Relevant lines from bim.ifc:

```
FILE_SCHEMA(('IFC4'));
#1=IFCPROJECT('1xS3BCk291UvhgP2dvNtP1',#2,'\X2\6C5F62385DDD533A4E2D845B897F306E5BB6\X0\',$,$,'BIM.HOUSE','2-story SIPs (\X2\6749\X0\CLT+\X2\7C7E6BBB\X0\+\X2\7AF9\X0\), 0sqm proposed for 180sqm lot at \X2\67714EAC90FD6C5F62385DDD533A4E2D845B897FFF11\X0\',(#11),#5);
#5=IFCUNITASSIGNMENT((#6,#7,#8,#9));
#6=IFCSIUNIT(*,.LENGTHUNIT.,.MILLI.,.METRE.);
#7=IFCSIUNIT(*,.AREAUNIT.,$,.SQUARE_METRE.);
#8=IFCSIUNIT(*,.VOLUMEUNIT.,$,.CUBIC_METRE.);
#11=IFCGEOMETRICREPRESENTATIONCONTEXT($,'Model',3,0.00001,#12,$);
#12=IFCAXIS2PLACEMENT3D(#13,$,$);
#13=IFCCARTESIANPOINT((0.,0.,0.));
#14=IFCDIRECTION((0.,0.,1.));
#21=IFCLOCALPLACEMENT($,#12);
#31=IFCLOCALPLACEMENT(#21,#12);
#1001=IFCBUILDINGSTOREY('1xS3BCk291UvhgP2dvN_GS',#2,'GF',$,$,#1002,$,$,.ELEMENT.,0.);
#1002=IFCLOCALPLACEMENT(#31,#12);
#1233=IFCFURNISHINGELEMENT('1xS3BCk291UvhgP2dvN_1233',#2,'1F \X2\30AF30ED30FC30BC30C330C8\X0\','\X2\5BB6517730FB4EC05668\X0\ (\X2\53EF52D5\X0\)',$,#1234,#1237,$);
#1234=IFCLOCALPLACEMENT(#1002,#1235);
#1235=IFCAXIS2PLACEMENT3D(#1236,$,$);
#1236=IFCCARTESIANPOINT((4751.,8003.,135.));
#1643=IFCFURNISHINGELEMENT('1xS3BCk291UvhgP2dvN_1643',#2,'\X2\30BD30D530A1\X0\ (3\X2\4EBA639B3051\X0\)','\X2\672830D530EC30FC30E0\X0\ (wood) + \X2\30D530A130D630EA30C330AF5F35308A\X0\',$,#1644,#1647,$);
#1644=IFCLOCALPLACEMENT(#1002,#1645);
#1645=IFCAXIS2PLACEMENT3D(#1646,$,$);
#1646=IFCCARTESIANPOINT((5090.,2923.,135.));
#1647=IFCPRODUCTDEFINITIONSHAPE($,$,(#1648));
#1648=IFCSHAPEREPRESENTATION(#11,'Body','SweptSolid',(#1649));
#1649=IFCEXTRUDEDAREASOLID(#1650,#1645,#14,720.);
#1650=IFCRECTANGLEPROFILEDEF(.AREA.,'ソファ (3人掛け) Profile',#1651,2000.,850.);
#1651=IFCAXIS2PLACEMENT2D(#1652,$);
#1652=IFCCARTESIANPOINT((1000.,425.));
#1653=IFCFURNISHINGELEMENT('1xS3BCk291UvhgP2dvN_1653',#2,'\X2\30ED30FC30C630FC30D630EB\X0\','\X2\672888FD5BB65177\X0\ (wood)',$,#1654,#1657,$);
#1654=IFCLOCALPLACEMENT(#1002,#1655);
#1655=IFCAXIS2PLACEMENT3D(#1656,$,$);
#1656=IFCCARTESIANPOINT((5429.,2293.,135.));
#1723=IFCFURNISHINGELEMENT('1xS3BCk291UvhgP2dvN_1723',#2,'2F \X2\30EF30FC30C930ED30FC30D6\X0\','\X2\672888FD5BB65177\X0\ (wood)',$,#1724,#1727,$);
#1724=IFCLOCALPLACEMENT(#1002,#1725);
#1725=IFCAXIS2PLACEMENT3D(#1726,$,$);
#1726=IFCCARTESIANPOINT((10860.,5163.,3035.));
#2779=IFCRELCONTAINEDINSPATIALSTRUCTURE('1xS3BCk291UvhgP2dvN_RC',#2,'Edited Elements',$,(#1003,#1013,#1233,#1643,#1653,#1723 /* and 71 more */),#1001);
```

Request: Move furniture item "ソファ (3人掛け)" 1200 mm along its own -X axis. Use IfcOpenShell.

```python
import ifcopenshell
import ifcopenshell.api.geometry
import ifcopenshell.util.placement
import ifcopenshell.util.unit

model = ifcopenshell.open("bim.ifc")
unit_scale = ifcopenshell.util.unit.calculate_unit_scale(model)

item = model.by_id(1643)
matrix = ifcopenshell.util.placement.get_local_placement(item.ObjectPlacement)
matrix[:3, 3] -= matrix[:3, 0] * 1.2 / unit_scale
ifcopenshell.api.geometry.edit_object_placement(model, product=item, matrix=matrix, is_si=False)

print(ifcopenshell.util.placement.get_local_placement(item.ObjectPlacement).round(3) + 0.0)

model.write("bim_edited.ifc")
```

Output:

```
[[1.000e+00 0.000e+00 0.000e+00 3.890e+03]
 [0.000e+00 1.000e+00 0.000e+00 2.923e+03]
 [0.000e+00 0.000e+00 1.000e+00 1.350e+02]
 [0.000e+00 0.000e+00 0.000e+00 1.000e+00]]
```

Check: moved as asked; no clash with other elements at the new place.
